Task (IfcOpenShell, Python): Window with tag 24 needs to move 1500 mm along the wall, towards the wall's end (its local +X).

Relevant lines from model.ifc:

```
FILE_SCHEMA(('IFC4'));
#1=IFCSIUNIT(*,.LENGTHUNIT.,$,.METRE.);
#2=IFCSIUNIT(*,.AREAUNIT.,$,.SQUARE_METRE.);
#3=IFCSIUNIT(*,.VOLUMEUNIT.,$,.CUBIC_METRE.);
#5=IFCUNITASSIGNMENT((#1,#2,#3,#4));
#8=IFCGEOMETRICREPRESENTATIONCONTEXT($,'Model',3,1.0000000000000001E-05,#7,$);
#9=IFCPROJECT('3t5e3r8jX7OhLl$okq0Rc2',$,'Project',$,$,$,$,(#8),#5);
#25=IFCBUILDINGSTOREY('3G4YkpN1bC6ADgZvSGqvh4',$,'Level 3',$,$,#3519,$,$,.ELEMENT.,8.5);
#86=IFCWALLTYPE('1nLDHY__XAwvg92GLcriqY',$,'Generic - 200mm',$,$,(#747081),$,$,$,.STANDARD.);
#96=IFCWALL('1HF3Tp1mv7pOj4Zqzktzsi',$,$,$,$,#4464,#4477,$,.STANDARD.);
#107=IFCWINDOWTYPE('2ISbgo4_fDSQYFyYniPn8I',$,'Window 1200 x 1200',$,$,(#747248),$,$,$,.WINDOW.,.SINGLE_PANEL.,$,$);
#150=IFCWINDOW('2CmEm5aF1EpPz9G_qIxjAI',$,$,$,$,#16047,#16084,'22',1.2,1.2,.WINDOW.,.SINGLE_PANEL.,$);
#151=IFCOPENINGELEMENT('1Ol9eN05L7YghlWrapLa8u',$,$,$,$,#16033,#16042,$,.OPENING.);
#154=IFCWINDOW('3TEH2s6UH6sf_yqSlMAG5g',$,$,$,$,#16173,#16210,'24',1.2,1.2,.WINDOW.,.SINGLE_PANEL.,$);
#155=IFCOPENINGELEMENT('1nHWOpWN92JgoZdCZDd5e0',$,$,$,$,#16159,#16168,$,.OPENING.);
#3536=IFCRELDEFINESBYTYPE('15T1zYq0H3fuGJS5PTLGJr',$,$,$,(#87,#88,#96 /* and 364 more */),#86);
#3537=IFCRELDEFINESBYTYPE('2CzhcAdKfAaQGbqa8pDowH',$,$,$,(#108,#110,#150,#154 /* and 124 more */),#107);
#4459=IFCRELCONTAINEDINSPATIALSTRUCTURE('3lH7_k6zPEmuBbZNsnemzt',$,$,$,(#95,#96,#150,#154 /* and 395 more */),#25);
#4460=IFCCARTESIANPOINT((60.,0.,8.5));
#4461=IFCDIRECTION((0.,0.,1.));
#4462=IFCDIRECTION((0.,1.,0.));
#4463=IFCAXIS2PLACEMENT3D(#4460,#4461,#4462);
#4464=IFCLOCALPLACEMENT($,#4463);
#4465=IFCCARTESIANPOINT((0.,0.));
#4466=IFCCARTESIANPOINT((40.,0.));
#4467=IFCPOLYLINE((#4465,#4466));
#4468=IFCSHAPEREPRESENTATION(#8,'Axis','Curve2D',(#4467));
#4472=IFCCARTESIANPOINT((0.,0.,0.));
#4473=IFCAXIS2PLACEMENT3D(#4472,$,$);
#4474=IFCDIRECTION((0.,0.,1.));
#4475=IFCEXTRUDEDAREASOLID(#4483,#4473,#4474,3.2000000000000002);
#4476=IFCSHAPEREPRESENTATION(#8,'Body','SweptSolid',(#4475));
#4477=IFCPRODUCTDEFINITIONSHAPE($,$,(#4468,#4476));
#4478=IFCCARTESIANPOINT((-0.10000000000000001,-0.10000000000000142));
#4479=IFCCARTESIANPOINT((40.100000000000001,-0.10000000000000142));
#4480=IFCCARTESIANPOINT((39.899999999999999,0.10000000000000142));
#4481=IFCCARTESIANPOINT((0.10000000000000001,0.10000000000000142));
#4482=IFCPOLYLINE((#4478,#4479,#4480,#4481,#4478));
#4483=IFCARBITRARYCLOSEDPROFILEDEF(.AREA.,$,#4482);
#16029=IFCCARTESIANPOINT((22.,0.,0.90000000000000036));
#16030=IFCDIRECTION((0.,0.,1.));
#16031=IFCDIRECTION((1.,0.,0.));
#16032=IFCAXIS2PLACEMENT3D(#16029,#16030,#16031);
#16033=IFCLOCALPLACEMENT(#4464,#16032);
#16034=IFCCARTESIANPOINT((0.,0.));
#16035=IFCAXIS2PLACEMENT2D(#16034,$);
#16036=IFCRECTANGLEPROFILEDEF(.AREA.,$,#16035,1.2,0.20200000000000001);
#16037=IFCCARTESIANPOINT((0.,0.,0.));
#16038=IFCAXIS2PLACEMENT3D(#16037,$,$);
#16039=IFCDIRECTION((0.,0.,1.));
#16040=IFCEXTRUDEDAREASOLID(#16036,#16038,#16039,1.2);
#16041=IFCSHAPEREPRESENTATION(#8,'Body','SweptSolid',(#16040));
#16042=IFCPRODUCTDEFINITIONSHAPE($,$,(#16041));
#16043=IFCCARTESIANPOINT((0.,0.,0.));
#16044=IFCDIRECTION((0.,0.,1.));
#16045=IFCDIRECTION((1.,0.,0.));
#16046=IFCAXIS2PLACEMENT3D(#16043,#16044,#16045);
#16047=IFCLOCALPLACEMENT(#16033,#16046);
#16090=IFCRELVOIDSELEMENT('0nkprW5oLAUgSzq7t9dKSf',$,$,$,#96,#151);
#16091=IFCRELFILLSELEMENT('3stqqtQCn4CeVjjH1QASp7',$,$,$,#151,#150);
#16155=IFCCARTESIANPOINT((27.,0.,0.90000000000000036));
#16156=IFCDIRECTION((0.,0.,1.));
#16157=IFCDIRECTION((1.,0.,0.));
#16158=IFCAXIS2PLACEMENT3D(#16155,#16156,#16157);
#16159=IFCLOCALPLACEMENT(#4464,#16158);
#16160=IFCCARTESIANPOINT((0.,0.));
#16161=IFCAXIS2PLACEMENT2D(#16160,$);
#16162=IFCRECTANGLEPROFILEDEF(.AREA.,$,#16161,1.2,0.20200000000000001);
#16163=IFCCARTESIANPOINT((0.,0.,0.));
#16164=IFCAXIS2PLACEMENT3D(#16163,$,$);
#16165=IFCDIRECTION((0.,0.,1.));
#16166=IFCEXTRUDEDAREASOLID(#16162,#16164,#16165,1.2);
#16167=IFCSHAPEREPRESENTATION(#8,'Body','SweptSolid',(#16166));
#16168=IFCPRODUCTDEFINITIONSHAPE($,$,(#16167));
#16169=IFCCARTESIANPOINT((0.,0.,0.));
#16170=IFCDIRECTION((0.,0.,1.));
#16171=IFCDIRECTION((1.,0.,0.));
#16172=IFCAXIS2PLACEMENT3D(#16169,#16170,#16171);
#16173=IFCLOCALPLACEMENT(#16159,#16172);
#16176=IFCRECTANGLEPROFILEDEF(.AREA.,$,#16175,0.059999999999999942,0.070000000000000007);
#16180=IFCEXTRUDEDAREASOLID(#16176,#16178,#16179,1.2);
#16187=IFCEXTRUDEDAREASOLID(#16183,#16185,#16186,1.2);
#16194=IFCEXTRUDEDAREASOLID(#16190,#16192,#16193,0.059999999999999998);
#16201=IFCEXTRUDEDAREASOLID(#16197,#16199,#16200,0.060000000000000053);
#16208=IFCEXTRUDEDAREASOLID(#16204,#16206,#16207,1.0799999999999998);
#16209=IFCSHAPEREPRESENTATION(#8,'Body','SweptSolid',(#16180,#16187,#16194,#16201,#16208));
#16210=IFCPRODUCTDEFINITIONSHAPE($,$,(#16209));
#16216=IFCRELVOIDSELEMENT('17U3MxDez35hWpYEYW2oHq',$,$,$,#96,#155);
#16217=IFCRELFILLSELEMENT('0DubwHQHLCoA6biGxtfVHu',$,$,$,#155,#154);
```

```python
import ifcopenshell
import ifcopenshell.api.geometry
import ifcopenshell.util.placement

model = ifcopenshell.open("model.ifc")

window = model.by_guid("3TEH2s6UH6sf_yqSlMAG5g")
opening = window.FillsVoids[0].RelatingOpeningElement
wall = opening.VoidsElements[0].RelatingBuildingElement

wall_matrix = ifcopenshell.util.placement.get_local_placement(wall.ObjectPlacement)
shift = wall_matrix[:3, 0] * 1.5
before = ifcopenshell.util.placement.get_local_placement(window.ObjectPlacement)[:3, 3].copy()

# The window is placed relative to its opening, so it follows when the opening moves.
matrix = ifcopenshell.util.placement.get_local_placement(opening.ObjectPlacement)
matrix[:3, 3] += shift
ifcopenshell.api.geometry.edit_object_placement(
    model, product=opening, matrix=matrix, is_si=False, should_transform_children=True
)

after = ifcopenshell.util.placement.get_local_placement(window.ObjectPlacement)[:3, 3]
print("window moved by", (after - before).round(3) + 0.0)

model.write("model_v2.ifc")
```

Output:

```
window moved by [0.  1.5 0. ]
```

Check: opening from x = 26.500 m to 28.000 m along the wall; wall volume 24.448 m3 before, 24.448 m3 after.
